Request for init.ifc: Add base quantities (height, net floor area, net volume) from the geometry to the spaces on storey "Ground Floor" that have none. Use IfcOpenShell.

First a look at what the model holds.

```python
import ifcopenshell
import ifcopenshell.util.element
import ifcopenshell.util.unit

model = ifcopenshell.open("init.ifc")
print(model.schema)
for unit_type in ("LENGTHUNIT", "AREAUNIT", "VOLUMEUNIT"):
    print(unit_type, ifcopenshell.util.unit.calculate_unit_scale(model, unit_type))
storey = next(s for s in model.by_type("IfcBuildingStorey") if s.Name == "Ground Floor")
spaces = [e for e in ifcopenshell.util.element.get_decomposition(storey) if e.is_a("IfcSpace")]
for e in sorted(spaces, key=lambda e: e.id()):
    print(e.id(), e.is_a(), e.Name, list(ifcopenshell.util.element.get_psets(e, qtos_only=True)), sep=" | ")
```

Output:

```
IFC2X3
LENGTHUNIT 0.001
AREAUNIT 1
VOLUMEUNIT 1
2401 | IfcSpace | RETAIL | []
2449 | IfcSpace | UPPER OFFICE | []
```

```python
import ifcopenshell
import ifcopenshell.api.pset
import ifcopenshell.geom
import ifcopenshell.util.element
import ifcopenshell.util.shape
import ifcopenshell.util.unit

model = ifcopenshell.open("init.ifc")
unit_scale = ifcopenshell.util.unit.calculate_unit_scale(model)
area_scale = ifcopenshell.util.unit.calculate_unit_scale(model, "AREAUNIT")
volume_scale = ifcopenshell.util.unit.calculate_unit_scale(model, "VOLUMEUNIT")
settings = ifcopenshell.geom.settings()

storey = next(s for s in model.by_type("IfcBuildingStorey") if s.Name == "Ground Floor")
spaces = [e for e in ifcopenshell.util.element.get_decomposition(storey) if e.is_a("IfcSpace")]

for e in sorted(spaces, key=lambda e: e.id()):
    if ifcopenshell.util.element.get_psets(e, qtos_only=True, should_inherit=False):
        continue
    # Geometry comes back in metres, in the element's own axes.
    shape = ifcopenshell.geom.create_shape(settings, e)
    values = {
        "Height": ifcopenshell.util.shape.get_z(shape.geometry) / unit_scale,
        "NetFloorArea": ifcopenshell.util.shape.get_footprint_area(shape.geometry) / area_scale,
        "NetVolume": ifcopenshell.util.shape.get_volume(shape.geometry) / volume_scale,
    }
    qto = ifcopenshell.api.pset.add_qto(model, product=e, name="BaseQuantities")
    ifcopenshell.api.pset.edit_qto(model, qto=qto, properties=values)
    print(e.id(), {k: round(v, 3) for k, v in values.items()})

model.write("init_rev.ifc")
```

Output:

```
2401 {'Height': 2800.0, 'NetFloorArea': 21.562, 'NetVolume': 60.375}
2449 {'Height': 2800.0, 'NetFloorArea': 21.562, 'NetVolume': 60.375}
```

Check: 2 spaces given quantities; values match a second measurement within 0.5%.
